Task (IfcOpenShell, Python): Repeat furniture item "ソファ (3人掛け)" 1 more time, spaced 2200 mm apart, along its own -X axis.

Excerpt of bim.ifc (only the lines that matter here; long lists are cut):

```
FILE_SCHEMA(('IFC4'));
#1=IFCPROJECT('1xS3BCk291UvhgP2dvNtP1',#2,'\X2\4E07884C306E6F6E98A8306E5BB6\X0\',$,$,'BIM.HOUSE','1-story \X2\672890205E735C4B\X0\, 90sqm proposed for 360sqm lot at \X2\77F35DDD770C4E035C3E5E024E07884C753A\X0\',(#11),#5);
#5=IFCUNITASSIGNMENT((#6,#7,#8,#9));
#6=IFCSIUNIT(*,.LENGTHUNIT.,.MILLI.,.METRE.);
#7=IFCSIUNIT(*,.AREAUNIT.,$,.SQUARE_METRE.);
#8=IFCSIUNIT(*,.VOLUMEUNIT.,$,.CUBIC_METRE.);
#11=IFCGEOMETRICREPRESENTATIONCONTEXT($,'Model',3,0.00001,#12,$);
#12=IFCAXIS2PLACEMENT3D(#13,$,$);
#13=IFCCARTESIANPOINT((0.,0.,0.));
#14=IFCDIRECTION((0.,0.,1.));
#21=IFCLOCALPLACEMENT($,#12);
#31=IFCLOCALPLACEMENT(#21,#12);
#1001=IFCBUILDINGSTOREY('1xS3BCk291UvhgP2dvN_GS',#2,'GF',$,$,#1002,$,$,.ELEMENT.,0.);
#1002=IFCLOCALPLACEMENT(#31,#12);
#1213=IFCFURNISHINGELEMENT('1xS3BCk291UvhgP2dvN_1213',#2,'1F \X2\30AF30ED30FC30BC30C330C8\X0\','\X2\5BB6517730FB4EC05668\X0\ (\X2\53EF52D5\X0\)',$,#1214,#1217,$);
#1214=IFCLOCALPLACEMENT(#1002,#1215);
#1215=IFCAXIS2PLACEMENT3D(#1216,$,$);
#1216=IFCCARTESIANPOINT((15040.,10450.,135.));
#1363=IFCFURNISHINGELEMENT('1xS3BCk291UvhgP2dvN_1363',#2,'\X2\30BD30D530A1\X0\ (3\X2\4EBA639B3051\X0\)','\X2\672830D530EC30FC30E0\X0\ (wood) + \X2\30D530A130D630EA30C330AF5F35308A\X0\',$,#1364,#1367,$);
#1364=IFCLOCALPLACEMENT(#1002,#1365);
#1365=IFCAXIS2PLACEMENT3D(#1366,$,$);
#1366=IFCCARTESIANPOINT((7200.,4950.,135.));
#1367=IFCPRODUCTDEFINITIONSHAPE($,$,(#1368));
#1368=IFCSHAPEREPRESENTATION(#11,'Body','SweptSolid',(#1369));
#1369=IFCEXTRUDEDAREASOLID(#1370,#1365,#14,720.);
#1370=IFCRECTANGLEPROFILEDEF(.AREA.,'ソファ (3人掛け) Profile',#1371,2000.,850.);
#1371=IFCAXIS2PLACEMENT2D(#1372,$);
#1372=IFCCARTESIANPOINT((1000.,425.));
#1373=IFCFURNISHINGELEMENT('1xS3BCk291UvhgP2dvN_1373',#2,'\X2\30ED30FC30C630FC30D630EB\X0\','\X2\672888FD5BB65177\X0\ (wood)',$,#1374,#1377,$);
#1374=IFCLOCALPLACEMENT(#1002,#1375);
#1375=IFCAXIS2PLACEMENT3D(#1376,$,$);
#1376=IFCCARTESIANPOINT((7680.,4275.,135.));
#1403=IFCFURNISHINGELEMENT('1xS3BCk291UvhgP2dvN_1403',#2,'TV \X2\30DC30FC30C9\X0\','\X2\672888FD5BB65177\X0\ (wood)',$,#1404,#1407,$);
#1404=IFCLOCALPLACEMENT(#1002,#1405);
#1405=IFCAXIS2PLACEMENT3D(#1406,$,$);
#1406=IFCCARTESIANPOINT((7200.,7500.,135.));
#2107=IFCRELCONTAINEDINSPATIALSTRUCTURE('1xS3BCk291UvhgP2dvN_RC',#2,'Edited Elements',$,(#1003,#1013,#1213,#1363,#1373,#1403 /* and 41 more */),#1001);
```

```python
import ifcopenshell
import ifcopenshell.api.geometry
import ifcopenshell.api.root
import ifcopenshell.util.element
import ifcopenshell.util.placement

model = ifcopenshell.open("bim.ifc")


def reuse_history(source, copy):
    """copy_class also copies each property set's owner history, people and application; keep the originals."""
    for rel in copy.IsDefinedBy:
        if rel.is_a("IfcRelDefinesByProperties") and (history := rel.RelatingPropertyDefinition.OwnerHistory):
            rel.RelatingPropertyDefinition.OwnerHistory = source.OwnerHistory
            ifcopenshell.util.element.remove_deep2(model, history)


source = model.by_guid("1xS3BCk291UvhgP2dvN_1363")
base = ifcopenshell.util.placement.get_local_placement(source.ObjectPlacement)
step = -base[:3, 0] * 2200.0

for i in range(1, 2):
    copy = ifcopenshell.api.root.copy_class(model, product=source)
    copy.Representation = ifcopenshell.util.element.copy_deep(
        model, source.Representation, exclude=["IfcGeometricRepresentationContext", "IfcRepresentationMap"]
    )
    reuse_history(source, copy)
    matrix = base.copy()
    matrix[:3, 3] += i * step
    print("added at", matrix[:3, 3].round(3) + 0.0)
    ifcopenshell.api.geometry.edit_object_placement(model, product=copy, matrix=matrix, is_si=False)

model.write("bim_edited.ifc")
```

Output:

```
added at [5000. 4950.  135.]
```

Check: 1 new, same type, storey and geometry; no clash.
